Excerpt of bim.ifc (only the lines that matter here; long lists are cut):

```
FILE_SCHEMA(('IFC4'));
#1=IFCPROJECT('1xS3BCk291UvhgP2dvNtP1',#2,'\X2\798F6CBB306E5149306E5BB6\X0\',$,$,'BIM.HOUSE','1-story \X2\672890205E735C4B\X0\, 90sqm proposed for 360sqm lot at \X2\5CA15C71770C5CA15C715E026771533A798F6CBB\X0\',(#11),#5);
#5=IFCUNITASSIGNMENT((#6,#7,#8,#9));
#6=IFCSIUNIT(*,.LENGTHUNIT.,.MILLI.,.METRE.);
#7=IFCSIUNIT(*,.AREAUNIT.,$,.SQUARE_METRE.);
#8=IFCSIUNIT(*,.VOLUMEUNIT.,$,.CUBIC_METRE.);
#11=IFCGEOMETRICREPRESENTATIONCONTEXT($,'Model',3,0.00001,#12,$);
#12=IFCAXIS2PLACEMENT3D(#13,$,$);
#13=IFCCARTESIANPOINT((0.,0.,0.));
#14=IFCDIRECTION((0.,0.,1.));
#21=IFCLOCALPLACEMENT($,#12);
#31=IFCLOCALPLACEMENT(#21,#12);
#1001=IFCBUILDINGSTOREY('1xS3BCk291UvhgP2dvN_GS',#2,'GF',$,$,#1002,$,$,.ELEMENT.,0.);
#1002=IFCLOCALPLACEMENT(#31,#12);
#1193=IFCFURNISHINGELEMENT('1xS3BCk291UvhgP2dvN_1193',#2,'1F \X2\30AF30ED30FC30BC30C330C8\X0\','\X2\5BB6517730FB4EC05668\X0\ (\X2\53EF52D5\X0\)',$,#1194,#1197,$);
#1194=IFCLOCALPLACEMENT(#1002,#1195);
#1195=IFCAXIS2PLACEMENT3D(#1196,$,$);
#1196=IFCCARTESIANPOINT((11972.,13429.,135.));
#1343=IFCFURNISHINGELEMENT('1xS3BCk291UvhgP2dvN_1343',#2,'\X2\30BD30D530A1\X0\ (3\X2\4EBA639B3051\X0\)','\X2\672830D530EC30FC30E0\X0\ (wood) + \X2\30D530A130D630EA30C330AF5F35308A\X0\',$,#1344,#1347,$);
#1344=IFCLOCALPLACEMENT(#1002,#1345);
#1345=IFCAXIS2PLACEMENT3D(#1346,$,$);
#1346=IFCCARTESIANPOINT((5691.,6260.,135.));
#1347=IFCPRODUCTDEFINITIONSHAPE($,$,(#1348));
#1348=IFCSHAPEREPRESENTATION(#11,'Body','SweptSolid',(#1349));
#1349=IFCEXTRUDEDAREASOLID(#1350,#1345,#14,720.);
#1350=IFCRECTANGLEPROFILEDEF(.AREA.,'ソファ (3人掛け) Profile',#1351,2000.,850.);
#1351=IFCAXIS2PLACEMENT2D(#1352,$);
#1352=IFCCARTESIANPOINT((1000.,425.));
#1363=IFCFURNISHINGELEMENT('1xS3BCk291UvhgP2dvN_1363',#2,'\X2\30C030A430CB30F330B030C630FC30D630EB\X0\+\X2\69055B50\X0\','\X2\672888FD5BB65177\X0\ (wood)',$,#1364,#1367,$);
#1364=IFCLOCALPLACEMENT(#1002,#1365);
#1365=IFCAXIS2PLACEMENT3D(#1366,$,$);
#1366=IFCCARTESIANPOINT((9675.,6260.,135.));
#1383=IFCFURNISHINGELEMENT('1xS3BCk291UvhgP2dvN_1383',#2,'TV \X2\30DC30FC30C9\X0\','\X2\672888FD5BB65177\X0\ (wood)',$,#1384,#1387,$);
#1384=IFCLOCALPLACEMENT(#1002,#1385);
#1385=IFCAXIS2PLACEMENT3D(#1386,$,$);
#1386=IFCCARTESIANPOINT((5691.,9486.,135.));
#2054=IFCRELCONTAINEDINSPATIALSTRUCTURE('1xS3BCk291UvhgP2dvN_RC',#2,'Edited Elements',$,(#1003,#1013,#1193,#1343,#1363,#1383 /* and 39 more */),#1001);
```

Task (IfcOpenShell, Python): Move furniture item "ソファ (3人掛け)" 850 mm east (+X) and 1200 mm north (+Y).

```python
import ifcopenshell
import ifcopenshell.api.geometry
import ifcopenshell.util.placement

model = ifcopenshell.open("bim.ifc")

item = model.by_guid("1xS3BCk291UvhgP2dvN_1343")
matrix = ifcopenshell.util.placement.get_local_placement(item.ObjectPlacement)
matrix[0, 3] += 850.0
matrix[1, 3] += 1200.0
ifcopenshell.api.geometry.edit_object_placement(model, product=item, matrix=matrix, is_si=False)

print(ifcopenshell.util.placement.get_local_placement(item.ObjectPlacement).round(3) + 0.0)

model.write("bim-out.ifc")
```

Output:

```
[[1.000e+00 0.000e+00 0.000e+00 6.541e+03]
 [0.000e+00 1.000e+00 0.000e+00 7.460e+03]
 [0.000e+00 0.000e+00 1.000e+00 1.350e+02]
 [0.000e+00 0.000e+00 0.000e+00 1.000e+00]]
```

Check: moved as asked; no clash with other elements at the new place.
